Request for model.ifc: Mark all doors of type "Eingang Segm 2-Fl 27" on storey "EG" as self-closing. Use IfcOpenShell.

First a look at what the model holds.

```python
import ifcopenshell
import ifcopenshell.util.element

model = ifcopenshell.open("model.ifc")
print(model.schema)
storey = next(s for s in model.by_type("IfcBuildingStorey") if s.Name == "EG")
doors = [e for e in ifcopenshell.util.element.get_decomposition(storey) if e.is_a("IfcDoor")]
seen = {}
for e in doors:
    element_type = ifcopenshell.util.element.get_type(e)
    key = (element_type.Name if element_type != e and element_type else None, ifcopenshell.util.element.get_pset(e, "Pset_DoorCommon", "SelfClosing"))
    seen[key] = seen.get(key, 0) + 1
for (name, value), count in sorted(seen.items(), key=str):
    print(count, "x", name, "|", value)
```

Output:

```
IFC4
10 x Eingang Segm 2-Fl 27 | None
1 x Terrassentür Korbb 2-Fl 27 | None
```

```python
import ifcopenshell
import ifcopenshell.api.pset
import ifcopenshell.util.element

model = ifcopenshell.open("model.ifc")

storey = next(s for s in model.by_type("IfcBuildingStorey") if s.Name == "EG")
doors = [e for e in ifcopenshell.util.element.get_decomposition(storey) if e.is_a("IfcDoor")]

count = 0
for e in doors:
    element_type = ifcopenshell.util.element.get_type(e)
    if element_type in (None, e) or element_type.Name != "Eingang Segm 2-Fl 27":
        continue
    # add_pset returns the element's existing set when there is one.
    pset = ifcopenshell.api.pset.add_pset(model, product=e, name="Pset_DoorCommon")
    ifcopenshell.api.pset.edit_pset(model, pset=pset, properties={"SelfClosing": True})
    count += 1

print(count, "doors updated")

model.write("model_rev.ifc")
```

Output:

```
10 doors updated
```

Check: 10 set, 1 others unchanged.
